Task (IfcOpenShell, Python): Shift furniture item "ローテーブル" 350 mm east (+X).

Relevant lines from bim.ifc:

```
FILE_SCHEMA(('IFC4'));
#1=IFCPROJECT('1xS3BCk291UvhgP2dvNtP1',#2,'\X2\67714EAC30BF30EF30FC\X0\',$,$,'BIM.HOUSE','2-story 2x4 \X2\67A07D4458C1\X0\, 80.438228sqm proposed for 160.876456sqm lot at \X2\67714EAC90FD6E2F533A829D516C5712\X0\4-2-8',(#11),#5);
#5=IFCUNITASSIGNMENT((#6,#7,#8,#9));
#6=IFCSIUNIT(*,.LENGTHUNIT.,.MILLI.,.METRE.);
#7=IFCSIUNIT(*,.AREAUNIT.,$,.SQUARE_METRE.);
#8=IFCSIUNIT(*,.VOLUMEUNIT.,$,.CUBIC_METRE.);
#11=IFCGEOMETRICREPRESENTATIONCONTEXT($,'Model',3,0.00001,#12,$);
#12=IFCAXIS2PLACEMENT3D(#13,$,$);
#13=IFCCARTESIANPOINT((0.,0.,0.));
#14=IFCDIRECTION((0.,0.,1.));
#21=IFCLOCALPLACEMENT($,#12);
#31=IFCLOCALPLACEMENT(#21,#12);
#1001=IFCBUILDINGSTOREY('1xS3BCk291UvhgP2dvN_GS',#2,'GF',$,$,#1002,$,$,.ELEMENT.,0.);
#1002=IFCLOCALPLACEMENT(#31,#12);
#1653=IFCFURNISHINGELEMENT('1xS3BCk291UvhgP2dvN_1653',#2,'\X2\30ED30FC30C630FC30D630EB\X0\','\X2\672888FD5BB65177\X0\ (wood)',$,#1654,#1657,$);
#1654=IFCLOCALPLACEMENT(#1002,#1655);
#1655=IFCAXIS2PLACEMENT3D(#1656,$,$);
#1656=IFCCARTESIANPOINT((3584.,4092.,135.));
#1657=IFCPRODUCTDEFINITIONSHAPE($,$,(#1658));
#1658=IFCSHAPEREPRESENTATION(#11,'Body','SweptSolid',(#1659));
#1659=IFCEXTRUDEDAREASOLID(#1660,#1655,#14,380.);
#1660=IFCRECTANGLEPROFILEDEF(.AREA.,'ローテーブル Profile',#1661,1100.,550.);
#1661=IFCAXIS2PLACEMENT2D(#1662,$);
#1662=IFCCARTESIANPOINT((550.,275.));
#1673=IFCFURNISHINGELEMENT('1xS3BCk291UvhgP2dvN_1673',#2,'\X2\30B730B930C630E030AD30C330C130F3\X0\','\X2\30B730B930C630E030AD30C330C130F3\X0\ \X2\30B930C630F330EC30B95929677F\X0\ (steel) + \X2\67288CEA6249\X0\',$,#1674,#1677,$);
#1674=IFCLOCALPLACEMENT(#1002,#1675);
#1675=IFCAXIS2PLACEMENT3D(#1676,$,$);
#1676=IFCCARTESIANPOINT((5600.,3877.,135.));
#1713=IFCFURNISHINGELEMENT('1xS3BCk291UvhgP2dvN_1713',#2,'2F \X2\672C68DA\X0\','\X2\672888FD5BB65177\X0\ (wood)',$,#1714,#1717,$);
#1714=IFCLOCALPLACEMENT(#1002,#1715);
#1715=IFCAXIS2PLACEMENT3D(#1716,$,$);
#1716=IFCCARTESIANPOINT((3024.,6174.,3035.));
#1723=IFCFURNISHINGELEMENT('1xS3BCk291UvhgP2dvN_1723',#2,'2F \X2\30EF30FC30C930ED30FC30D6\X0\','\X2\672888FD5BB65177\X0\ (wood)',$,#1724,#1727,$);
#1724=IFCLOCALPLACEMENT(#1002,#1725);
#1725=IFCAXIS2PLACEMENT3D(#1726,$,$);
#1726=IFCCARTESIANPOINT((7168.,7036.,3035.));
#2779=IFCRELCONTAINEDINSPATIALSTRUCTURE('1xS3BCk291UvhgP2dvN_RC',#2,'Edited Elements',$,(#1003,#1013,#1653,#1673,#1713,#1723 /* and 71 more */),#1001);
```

```python
import ifcopenshell
import ifcopenshell.api.geometry
import ifcopenshell.util.placement

model = ifcopenshell.open("bim.ifc")

item = model.by_guid("1xS3BCk291UvhgP2dvN_1653")
matrix = ifcopenshell.util.placement.get_local_placement(item.ObjectPlacement)
matrix[0, 3] += 350.0
ifcopenshell.api.geometry.edit_object_placement(model, product=item, matrix=matrix, is_si=False)

print(ifcopenshell.util.placement.get_local_placement(item.ObjectPlacement).round(3) + 0.0)

model.write("bim_rev.ifc")
```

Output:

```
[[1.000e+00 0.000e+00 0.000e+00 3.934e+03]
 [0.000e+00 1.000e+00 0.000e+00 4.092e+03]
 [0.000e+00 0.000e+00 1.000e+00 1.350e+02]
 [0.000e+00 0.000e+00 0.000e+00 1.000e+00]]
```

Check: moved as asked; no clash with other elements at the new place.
